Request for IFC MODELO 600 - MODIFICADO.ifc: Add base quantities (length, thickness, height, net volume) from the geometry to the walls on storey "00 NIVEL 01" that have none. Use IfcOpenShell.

First a look at what the model holds.

```python
import ifcopenshell
import ifcopenshell.util.element
import ifcopenshell.util.unit

model = ifcopenshell.open("IFC MODELO 600 - MODIFICADO.ifc")
print(model.schema)
for unit_type in ("LENGTHUNIT", "AREAUNIT", "VOLUMEUNIT"):
    print(unit_type, ifcopenshell.util.unit.calculate_unit_scale(model, unit_type))
storey = next(s for s in model.by_type("IfcBuildingStorey") if s.Name == "00 NIVEL 01")
walls = [e for e in ifcopenshell.util.element.get_decomposition(storey) if e.is_a("IfcWall")]
for e in sorted(walls, key=lambda e: e.id()):
    print(e.id(), e.is_a(), e.Name, list(ifcopenshell.util.element.get_psets(e, qtos_only=True)), sep=" | ")
```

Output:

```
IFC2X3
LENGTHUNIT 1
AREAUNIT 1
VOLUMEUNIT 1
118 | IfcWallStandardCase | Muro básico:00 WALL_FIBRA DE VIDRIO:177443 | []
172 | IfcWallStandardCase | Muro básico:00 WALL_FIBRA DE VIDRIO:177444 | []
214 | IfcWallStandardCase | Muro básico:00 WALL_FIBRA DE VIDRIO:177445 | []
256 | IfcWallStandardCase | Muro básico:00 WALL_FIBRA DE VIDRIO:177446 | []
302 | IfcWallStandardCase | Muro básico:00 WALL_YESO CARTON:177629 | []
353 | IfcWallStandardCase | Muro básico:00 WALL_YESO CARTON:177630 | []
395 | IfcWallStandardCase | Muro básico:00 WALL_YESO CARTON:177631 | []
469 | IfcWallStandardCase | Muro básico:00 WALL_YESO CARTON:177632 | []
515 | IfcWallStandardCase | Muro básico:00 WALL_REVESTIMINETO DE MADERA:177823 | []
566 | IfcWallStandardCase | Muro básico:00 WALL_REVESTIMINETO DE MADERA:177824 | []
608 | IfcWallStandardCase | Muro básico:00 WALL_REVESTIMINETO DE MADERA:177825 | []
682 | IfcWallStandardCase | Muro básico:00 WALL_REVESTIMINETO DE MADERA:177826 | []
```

```python
import ifcopenshell
import ifcopenshell.api.pset
import ifcopenshell.geom
import ifcopenshell.util.element
import ifcopenshell.util.shape
import ifcopenshell.util.unit

model = ifcopenshell.open("IFC MODELO 600 - MODIFICADO.ifc")
unit_scale = ifcopenshell.util.unit.calculate_unit_scale(model)
volume_scale = ifcopenshell.util.unit.calculate_unit_scale(model, "VOLUMEUNIT")
settings = ifcopenshell.geom.settings()

storey = next(s for s in model.by_type("IfcBuildingStorey") if s.Name == "00 NIVEL 01")
walls = [e for e in ifcopenshell.util.element.get_decomposition(storey) if e.is_a("IfcWall")]

for e in sorted(walls, key=lambda e: e.id()):
    if ifcopenshell.util.element.get_psets(e, qtos_only=True, should_inherit=False):
        continue
    # Geometry comes back in metres, in the element's own axes.
    shape = ifcopenshell.geom.create_shape(settings, e)
    values = {
        "Length": ifcopenshell.util.shape.get_x(shape.geometry) / unit_scale,
        "Width": ifcopenshell.util.shape.get_y(shape.geometry) / unit_scale,
        "Height": ifcopenshell.util.shape.get_z(shape.geometry) / unit_scale,
        "NetVolume": ifcopenshell.util.shape.get_volume(shape.geometry) / volume_scale,
    }
    qto = ifcopenshell.api.pset.add_qto(model, product=e, name="BaseQuantities")
    ifcopenshell.api.pset.edit_qto(model, qto=qto, properties=values)
    print(e.id(), {k: round(v, 3) for k, v in values.items()})

model.write("IFC MODELO 600 - MODIFICADO_rev.ifc")
```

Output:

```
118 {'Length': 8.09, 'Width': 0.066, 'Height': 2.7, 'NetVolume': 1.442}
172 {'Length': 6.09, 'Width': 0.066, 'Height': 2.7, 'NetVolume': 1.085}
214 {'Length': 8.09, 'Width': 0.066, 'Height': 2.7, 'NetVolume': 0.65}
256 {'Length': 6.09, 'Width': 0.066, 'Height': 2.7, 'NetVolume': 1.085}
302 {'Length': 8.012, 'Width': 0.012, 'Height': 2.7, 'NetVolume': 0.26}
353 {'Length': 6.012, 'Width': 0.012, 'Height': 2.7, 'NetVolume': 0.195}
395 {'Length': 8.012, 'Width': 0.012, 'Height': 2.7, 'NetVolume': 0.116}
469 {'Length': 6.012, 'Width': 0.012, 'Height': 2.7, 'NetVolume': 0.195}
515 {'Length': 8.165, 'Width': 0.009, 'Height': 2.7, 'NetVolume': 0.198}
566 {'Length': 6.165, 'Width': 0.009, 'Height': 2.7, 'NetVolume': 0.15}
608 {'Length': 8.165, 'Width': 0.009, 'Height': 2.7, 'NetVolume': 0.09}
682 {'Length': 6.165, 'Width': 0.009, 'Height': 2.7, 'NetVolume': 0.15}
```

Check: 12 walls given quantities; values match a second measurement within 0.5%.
